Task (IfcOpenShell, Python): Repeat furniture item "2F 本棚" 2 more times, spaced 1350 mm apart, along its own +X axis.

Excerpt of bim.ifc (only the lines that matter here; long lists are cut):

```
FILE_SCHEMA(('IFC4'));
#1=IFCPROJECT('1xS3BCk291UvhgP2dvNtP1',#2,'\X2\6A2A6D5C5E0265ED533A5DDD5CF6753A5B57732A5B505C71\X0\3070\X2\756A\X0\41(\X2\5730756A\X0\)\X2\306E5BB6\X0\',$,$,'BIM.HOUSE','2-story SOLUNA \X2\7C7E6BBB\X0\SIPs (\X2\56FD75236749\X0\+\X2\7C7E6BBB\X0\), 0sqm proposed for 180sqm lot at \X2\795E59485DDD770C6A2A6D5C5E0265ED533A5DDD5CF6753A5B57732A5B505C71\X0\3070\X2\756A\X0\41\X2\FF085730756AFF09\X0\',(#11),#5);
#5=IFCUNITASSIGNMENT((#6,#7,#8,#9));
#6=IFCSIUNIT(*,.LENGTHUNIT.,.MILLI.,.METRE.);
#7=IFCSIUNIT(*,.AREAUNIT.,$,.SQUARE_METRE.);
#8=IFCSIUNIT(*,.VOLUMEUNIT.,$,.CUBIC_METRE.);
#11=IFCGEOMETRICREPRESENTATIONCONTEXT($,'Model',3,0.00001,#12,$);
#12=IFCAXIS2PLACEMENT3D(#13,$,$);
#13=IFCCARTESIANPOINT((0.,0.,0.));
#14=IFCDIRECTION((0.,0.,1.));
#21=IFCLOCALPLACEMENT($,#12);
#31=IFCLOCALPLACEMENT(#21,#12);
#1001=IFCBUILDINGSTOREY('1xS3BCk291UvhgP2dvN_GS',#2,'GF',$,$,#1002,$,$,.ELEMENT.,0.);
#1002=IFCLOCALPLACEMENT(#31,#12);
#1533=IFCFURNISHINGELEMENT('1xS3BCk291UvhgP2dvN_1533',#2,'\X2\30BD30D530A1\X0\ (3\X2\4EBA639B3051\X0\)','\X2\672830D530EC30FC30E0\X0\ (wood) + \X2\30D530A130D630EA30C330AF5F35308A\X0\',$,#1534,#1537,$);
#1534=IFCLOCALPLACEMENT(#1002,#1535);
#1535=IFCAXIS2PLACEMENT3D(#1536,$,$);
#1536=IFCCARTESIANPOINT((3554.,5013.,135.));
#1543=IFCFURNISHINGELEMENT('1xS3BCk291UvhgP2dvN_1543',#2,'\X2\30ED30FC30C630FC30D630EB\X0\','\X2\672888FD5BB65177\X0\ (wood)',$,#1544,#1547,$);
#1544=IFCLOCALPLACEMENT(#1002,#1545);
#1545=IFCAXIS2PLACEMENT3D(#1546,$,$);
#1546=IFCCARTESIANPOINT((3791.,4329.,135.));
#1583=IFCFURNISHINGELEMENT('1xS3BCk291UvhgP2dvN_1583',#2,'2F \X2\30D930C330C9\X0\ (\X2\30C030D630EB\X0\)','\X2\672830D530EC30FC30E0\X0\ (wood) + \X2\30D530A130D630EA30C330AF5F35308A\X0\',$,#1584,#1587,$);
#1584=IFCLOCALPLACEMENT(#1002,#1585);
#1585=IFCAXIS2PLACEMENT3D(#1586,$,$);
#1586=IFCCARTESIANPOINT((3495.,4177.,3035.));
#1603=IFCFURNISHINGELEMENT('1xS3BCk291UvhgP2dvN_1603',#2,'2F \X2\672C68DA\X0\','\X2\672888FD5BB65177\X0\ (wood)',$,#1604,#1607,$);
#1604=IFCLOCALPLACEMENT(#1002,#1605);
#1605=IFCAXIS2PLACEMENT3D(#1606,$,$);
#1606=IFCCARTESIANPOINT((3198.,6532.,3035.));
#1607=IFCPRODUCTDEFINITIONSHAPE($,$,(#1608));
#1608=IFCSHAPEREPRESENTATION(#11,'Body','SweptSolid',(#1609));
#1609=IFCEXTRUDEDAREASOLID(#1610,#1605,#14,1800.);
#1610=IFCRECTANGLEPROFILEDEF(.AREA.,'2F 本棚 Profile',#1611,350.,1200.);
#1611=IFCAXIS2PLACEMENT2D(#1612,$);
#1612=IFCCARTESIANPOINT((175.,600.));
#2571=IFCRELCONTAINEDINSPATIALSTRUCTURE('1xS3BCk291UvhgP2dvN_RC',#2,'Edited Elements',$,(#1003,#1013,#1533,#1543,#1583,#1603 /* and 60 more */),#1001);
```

```python
import ifcopenshell
import ifcopenshell.api.geometry
import ifcopenshell.api.root
import ifcopenshell.util.element
import ifcopenshell.util.placement
import ifcopenshell.util.unit

model = ifcopenshell.open("bim.ifc")
unit_scale = ifcopenshell.util.unit.calculate_unit_scale(model)


def reuse_history(source, copy):
    """copy_class also copies each property set's owner history, people and application; keep the originals."""
    for rel in copy.IsDefinedBy:
        if rel.is_a("IfcRelDefinesByProperties") and (history := rel.RelatingPropertyDefinition.OwnerHistory):
            rel.RelatingPropertyDefinition.OwnerHistory = source.OwnerHistory
            ifcopenshell.util.element.remove_deep2(model, history)


source = model.by_guid("1xS3BCk291UvhgP2dvN_1603")
base = ifcopenshell.util.placement.get_local_placement(source.ObjectPlacement)
step = base[:3, 0] * 1.35 / unit_scale

for i in range(1, 3):
    copy = ifcopenshell.api.root.copy_class(model, product=source)
    copy.Representation = ifcopenshell.util.element.copy_deep(
        model, source.Representation, exclude=["IfcGeometricRepresentationContext", "IfcRepresentationMap"]
    )
    reuse_history(source, copy)
    matrix = base.copy()
    matrix[:3, 3] += i * step
    print("added at", matrix[:3, 3].round(3) + 0.0)
    ifcopenshell.api.geometry.edit_object_placement(model, product=copy, matrix=matrix, is_si=False)

model.write("bim_rev.ifc")
```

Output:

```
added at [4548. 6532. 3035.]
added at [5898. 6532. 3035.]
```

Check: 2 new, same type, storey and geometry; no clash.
